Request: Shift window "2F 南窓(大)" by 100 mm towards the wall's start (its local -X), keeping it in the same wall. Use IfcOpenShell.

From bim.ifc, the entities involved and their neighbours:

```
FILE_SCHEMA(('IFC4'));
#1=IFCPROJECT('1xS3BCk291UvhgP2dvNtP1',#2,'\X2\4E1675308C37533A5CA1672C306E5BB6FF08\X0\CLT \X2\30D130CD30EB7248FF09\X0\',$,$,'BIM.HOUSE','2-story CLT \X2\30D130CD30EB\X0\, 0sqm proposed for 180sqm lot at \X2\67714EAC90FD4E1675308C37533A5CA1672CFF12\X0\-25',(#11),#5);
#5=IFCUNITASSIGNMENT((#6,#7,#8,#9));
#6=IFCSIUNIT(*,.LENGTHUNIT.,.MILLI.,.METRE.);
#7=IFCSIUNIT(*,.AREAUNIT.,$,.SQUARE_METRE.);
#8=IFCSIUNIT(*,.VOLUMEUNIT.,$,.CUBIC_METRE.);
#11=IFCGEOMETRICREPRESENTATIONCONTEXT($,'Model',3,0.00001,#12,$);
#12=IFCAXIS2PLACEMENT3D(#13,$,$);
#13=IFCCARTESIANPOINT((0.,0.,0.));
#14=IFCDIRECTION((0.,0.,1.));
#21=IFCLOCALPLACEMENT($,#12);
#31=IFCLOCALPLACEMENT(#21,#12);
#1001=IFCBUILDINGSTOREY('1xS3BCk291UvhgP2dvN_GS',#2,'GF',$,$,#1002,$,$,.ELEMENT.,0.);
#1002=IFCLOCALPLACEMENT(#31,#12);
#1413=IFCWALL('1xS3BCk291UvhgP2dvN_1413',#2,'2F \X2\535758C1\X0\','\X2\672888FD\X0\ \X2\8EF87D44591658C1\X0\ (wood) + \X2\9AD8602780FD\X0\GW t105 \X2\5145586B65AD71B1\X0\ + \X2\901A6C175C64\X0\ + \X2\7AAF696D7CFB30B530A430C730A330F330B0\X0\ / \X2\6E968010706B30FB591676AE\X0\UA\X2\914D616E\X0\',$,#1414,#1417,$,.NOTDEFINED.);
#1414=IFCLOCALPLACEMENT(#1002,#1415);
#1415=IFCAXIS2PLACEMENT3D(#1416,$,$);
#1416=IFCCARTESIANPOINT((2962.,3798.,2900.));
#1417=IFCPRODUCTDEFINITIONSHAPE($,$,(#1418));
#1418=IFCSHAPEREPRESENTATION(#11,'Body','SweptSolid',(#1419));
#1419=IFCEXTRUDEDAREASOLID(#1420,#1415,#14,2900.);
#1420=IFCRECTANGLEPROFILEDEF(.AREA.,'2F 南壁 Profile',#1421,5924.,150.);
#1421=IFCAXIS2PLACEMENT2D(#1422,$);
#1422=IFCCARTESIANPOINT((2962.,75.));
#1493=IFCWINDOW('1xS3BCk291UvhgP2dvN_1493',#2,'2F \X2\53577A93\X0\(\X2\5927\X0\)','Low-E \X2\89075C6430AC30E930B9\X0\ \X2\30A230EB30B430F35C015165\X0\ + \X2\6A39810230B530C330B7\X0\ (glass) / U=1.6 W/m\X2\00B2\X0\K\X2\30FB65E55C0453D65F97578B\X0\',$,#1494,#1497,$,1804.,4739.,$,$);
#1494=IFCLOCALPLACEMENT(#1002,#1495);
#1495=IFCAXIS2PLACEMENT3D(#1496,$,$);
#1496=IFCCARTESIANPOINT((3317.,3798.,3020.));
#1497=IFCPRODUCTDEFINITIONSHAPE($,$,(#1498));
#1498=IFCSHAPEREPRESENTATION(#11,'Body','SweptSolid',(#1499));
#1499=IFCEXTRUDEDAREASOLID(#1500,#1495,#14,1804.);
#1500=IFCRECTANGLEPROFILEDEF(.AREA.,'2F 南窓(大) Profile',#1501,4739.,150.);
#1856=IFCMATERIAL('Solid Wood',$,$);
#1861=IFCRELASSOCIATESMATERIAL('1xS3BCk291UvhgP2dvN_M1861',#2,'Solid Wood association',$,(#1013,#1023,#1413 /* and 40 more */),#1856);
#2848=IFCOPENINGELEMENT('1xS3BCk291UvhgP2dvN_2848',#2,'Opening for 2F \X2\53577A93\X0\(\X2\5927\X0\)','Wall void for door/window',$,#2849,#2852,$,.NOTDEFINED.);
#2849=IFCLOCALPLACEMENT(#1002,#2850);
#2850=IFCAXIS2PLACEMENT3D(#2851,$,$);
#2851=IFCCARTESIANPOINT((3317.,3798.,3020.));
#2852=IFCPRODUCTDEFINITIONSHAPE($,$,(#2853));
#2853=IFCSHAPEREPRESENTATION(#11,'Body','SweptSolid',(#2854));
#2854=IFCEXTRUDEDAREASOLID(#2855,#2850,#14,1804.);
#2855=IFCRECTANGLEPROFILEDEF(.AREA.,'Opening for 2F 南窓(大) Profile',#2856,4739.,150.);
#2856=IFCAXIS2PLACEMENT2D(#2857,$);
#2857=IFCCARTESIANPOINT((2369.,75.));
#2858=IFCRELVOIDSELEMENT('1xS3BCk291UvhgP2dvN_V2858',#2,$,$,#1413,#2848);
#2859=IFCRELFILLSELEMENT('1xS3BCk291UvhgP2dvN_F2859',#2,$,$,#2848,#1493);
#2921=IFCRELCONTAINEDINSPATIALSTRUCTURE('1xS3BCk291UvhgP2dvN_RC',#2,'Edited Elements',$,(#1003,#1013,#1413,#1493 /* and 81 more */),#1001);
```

```python
import ifcopenshell
import ifcopenshell.api.geometry
import ifcopenshell.util.placement

model = ifcopenshell.open("bim.ifc")

window = model.by_guid("1xS3BCk291UvhgP2dvN_1493")
opening = window.FillsVoids[0].RelatingOpeningElement
wall = opening.VoidsElements[0].RelatingBuildingElement

wall_matrix = ifcopenshell.util.placement.get_local_placement(wall.ObjectPlacement)
shift = wall_matrix[:3, 0] * -100.0
before = ifcopenshell.util.placement.get_local_placement(window.ObjectPlacement)[:3, 3].copy()

# The window is not placed relative to its opening, so move both.
for product in (opening, window):
    matrix = ifcopenshell.util.placement.get_local_placement(product.ObjectPlacement)
    matrix[:3, 3] += shift
    ifcopenshell.api.geometry.edit_object_placement(model, product=product, matrix=matrix, is_si=False)

after = ifcopenshell.util.placement.get_local_placement(window.ObjectPlacement)[:3, 3]
print("window moved by", (after - before).round(3) + 0.0)

model.write("bim-out.ifc")
```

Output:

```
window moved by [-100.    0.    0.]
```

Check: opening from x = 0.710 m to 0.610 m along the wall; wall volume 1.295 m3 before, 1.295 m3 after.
